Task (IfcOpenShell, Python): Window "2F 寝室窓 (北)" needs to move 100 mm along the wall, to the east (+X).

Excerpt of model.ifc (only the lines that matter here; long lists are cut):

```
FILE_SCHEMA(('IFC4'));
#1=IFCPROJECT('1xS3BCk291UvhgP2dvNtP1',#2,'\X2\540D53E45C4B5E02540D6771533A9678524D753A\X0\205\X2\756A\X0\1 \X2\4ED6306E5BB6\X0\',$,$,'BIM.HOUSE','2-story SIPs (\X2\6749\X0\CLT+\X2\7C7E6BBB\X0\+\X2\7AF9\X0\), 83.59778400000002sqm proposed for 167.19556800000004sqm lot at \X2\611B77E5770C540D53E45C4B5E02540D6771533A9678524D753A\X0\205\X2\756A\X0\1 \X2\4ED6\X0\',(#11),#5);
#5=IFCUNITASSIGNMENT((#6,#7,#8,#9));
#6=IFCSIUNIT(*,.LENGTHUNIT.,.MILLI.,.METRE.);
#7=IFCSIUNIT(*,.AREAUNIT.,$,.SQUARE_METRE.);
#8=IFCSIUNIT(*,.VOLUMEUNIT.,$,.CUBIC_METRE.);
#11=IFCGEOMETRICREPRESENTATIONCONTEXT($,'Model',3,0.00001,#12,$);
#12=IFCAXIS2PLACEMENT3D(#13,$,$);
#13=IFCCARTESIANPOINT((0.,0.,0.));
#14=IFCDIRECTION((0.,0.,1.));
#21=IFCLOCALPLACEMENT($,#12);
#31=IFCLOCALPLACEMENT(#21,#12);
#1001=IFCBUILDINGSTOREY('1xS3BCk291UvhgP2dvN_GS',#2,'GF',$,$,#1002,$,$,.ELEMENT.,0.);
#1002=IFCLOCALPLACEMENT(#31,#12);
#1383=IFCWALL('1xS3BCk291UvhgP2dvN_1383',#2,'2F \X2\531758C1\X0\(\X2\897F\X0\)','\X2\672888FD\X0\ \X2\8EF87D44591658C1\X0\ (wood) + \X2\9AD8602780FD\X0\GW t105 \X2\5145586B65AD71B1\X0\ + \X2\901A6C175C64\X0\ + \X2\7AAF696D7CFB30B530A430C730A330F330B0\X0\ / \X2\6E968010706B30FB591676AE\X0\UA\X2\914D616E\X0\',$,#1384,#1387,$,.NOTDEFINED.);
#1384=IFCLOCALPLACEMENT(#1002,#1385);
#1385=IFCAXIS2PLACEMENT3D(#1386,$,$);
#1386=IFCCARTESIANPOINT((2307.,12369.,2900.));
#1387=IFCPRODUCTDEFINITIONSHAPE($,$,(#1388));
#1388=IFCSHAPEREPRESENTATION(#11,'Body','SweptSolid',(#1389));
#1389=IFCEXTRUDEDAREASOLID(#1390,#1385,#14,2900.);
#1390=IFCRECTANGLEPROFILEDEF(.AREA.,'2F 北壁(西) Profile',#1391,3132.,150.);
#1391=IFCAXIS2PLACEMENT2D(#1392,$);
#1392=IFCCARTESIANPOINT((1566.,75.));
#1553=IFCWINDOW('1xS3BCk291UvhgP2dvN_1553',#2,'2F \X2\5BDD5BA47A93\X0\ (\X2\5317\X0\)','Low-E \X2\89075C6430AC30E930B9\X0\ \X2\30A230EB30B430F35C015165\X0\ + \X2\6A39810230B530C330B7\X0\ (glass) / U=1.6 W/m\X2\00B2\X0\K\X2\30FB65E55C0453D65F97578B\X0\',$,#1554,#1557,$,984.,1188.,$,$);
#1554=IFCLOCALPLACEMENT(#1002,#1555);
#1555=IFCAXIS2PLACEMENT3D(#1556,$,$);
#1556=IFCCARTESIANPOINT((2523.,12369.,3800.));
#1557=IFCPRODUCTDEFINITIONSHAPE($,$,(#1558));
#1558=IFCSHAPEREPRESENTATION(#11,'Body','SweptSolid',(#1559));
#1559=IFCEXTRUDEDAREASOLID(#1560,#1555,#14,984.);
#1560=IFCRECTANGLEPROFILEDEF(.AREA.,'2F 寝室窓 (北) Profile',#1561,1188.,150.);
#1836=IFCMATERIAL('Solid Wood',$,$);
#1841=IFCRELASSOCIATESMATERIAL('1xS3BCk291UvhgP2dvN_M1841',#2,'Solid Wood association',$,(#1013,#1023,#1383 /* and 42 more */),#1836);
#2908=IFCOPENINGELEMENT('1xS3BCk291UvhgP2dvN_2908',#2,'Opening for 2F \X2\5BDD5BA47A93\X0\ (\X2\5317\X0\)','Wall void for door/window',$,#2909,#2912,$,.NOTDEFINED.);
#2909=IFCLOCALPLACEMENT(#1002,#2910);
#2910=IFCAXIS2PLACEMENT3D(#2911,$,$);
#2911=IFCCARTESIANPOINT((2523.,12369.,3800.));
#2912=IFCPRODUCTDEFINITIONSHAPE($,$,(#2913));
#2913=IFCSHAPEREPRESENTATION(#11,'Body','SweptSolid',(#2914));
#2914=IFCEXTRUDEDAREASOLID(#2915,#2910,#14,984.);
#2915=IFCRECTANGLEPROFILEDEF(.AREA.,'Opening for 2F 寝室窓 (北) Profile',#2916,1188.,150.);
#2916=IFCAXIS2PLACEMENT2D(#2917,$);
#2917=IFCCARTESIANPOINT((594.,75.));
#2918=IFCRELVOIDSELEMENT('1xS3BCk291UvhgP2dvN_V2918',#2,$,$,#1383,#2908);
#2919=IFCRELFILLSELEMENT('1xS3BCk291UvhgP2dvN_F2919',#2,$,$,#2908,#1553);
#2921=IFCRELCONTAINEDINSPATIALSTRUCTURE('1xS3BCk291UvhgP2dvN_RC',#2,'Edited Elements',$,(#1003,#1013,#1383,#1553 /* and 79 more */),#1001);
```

```python
import ifcopenshell
import ifcopenshell.api.geometry
import ifcopenshell.util.placement
import ifcopenshell.util.unit

model = ifcopenshell.open("model.ifc")
unit_scale = ifcopenshell.util.unit.calculate_unit_scale(model)

window = model.by_id(1553)
opening = window.FillsVoids[0].RelatingOpeningElement
wall = opening.VoidsElements[0].RelatingBuildingElement

wall_matrix = ifcopenshell.util.placement.get_local_placement(wall.ObjectPlacement)
shift = wall_matrix[:3, 0] * 0.1 / unit_scale
before = ifcopenshell.util.placement.get_local_placement(window.ObjectPlacement)[:3, 3].copy()

# The window is not placed relative to its opening, so move both.
for product in (opening, window):
    matrix = ifcopenshell.util.placement.get_local_placement(product.ObjectPlacement)
    matrix[:3, 3] += shift
    ifcopenshell.api.geometry.edit_object_placement(model, product=product, matrix=matrix, is_si=False)

after = ifcopenshell.util.placement.get_local_placement(window.ObjectPlacement)[:3, 3]
print("window moved by", (after - before).round(3) + 0.0)

model.write("model-out.ifc")
```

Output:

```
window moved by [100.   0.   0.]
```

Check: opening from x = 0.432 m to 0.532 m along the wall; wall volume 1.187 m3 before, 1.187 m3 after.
